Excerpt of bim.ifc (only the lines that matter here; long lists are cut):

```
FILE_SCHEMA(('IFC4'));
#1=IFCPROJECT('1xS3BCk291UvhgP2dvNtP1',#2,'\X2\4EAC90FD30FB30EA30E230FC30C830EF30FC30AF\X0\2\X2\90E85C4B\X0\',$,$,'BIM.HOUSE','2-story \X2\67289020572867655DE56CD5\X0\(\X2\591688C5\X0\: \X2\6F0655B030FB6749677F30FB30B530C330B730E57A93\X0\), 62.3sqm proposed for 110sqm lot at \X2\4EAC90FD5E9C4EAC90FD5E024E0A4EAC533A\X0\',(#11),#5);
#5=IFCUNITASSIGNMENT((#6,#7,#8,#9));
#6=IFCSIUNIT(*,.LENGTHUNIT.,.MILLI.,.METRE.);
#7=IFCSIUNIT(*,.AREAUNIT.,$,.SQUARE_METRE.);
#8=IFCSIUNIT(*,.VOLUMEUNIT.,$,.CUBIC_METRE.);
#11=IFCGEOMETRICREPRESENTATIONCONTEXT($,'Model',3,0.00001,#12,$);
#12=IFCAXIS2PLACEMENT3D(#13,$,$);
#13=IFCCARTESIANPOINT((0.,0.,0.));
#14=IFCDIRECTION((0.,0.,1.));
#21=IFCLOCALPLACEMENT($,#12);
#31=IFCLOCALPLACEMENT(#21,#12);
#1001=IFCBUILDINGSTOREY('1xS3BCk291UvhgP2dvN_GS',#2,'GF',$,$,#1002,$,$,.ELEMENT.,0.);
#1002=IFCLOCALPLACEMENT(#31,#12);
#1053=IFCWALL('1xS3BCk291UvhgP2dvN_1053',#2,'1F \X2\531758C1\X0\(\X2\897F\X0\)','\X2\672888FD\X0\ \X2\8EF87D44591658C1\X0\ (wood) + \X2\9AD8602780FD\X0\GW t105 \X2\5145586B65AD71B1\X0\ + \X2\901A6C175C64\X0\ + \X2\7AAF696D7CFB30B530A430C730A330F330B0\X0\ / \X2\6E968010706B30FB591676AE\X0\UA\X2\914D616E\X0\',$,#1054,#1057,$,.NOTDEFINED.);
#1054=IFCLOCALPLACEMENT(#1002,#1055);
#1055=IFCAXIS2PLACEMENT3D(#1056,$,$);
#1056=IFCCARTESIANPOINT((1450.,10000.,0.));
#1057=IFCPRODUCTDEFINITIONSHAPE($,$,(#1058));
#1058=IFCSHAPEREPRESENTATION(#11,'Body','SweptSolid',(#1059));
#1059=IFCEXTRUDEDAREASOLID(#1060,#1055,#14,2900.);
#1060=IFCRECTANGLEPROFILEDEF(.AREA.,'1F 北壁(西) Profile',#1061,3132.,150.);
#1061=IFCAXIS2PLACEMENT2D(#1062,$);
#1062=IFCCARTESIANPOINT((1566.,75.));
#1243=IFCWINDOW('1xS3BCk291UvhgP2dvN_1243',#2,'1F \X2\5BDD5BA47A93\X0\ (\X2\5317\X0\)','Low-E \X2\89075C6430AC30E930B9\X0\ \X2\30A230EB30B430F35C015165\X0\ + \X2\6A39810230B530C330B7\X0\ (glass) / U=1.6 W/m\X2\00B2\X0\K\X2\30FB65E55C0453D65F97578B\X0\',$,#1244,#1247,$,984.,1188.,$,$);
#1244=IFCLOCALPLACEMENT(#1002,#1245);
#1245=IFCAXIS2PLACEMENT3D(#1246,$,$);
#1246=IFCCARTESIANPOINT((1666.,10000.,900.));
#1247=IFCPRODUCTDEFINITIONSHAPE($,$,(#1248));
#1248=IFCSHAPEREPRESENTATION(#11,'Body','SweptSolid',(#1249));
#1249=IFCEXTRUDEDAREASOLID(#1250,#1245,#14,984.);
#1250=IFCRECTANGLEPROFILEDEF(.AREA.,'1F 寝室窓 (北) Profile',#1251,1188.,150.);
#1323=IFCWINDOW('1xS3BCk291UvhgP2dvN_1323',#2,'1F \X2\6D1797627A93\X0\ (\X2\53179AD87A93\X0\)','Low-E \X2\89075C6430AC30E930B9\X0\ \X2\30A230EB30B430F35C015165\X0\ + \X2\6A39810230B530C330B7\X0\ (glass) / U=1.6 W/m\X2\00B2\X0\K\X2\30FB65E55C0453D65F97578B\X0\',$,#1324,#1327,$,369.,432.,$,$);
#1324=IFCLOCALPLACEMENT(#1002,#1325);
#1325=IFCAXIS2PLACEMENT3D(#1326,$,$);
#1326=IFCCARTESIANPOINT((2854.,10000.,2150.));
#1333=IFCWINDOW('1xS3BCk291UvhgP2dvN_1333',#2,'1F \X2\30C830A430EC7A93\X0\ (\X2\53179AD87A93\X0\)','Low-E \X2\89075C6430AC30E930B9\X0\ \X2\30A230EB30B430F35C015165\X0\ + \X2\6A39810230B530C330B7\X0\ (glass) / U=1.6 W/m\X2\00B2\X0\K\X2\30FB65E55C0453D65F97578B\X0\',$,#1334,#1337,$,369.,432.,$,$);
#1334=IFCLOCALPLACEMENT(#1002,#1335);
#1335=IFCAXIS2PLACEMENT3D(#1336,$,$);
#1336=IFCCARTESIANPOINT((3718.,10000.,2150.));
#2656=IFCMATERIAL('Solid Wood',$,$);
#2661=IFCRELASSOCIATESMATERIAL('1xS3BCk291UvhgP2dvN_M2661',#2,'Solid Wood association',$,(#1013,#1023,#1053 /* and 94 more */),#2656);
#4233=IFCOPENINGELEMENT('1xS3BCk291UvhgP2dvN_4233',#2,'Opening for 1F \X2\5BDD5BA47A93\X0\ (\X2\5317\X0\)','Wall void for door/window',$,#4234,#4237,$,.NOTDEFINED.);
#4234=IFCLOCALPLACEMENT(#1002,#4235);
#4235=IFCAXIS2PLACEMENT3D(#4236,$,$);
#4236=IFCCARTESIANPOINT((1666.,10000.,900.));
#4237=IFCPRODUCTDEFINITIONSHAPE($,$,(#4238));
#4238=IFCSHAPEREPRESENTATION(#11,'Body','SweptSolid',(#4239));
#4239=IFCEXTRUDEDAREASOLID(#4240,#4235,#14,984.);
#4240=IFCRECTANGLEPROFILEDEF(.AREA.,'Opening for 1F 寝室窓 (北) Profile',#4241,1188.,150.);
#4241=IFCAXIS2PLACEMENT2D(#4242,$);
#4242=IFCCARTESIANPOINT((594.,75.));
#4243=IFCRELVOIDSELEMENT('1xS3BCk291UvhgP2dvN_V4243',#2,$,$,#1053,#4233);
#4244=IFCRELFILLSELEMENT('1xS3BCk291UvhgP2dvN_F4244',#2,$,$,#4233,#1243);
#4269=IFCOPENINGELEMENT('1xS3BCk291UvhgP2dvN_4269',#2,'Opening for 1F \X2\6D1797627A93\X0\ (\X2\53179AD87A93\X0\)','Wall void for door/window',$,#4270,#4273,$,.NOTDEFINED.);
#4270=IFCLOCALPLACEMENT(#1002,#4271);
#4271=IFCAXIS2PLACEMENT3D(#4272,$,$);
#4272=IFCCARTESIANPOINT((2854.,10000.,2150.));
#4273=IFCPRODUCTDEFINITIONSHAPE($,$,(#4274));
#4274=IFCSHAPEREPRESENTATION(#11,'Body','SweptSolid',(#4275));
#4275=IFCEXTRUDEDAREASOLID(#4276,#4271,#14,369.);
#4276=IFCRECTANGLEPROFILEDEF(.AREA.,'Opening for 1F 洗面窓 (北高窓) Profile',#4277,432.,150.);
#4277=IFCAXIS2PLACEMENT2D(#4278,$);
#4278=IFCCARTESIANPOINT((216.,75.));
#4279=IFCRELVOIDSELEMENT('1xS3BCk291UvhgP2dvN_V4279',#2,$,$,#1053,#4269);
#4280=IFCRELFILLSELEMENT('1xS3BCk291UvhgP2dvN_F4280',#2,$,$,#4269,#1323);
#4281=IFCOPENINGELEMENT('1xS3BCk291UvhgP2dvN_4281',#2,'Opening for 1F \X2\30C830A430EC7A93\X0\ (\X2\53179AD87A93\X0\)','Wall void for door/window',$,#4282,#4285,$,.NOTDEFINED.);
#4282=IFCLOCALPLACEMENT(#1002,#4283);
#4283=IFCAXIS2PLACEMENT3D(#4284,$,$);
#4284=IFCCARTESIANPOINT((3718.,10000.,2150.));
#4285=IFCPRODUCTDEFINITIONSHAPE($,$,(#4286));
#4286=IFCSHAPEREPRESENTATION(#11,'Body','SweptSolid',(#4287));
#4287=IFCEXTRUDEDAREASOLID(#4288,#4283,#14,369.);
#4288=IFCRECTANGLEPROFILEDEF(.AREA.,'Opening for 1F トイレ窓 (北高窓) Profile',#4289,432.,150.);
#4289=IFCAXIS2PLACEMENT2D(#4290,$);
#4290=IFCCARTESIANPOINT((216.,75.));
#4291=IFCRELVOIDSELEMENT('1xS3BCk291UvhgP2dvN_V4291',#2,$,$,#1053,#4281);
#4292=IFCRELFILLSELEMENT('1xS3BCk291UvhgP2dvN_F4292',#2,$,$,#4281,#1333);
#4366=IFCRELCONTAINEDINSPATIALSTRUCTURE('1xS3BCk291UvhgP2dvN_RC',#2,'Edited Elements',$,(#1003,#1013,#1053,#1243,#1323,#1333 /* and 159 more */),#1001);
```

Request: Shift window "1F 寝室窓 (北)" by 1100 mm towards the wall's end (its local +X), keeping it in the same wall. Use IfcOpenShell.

```python
import ifcopenshell
import ifcopenshell.api.geometry
import ifcopenshell.util.placement

model = ifcopenshell.open("bim.ifc")

window = model.by_guid("1xS3BCk291UvhgP2dvN_1243")
opening = window.FillsVoids[0].RelatingOpeningElement
wall = opening.VoidsElements[0].RelatingBuildingElement

wall_matrix = ifcopenshell.util.placement.get_local_placement(wall.ObjectPlacement)
shift = wall_matrix[:3, 0] * 1100.0
before = ifcopenshell.util.placement.get_local_placement(window.ObjectPlacement)[:3, 3].copy()

# The window is not placed relative to its opening, so move both.
for product in (opening, window):
    matrix = ifcopenshell.util.placement.get_local_placement(product.ObjectPlacement)
    matrix[:3, 3] += shift
    ifcopenshell.api.geometry.edit_object_placement(model, product=product, matrix=matrix, is_si=False)

after = ifcopenshell.util.placement.get_local_placement(window.ObjectPlacement)[:3, 3]
print("window moved by", (after - before).round(3) + 0.0)

model.write("bim-out.ifc")
```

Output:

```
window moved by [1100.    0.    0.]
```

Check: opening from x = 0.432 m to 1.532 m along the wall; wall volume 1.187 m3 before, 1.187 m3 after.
